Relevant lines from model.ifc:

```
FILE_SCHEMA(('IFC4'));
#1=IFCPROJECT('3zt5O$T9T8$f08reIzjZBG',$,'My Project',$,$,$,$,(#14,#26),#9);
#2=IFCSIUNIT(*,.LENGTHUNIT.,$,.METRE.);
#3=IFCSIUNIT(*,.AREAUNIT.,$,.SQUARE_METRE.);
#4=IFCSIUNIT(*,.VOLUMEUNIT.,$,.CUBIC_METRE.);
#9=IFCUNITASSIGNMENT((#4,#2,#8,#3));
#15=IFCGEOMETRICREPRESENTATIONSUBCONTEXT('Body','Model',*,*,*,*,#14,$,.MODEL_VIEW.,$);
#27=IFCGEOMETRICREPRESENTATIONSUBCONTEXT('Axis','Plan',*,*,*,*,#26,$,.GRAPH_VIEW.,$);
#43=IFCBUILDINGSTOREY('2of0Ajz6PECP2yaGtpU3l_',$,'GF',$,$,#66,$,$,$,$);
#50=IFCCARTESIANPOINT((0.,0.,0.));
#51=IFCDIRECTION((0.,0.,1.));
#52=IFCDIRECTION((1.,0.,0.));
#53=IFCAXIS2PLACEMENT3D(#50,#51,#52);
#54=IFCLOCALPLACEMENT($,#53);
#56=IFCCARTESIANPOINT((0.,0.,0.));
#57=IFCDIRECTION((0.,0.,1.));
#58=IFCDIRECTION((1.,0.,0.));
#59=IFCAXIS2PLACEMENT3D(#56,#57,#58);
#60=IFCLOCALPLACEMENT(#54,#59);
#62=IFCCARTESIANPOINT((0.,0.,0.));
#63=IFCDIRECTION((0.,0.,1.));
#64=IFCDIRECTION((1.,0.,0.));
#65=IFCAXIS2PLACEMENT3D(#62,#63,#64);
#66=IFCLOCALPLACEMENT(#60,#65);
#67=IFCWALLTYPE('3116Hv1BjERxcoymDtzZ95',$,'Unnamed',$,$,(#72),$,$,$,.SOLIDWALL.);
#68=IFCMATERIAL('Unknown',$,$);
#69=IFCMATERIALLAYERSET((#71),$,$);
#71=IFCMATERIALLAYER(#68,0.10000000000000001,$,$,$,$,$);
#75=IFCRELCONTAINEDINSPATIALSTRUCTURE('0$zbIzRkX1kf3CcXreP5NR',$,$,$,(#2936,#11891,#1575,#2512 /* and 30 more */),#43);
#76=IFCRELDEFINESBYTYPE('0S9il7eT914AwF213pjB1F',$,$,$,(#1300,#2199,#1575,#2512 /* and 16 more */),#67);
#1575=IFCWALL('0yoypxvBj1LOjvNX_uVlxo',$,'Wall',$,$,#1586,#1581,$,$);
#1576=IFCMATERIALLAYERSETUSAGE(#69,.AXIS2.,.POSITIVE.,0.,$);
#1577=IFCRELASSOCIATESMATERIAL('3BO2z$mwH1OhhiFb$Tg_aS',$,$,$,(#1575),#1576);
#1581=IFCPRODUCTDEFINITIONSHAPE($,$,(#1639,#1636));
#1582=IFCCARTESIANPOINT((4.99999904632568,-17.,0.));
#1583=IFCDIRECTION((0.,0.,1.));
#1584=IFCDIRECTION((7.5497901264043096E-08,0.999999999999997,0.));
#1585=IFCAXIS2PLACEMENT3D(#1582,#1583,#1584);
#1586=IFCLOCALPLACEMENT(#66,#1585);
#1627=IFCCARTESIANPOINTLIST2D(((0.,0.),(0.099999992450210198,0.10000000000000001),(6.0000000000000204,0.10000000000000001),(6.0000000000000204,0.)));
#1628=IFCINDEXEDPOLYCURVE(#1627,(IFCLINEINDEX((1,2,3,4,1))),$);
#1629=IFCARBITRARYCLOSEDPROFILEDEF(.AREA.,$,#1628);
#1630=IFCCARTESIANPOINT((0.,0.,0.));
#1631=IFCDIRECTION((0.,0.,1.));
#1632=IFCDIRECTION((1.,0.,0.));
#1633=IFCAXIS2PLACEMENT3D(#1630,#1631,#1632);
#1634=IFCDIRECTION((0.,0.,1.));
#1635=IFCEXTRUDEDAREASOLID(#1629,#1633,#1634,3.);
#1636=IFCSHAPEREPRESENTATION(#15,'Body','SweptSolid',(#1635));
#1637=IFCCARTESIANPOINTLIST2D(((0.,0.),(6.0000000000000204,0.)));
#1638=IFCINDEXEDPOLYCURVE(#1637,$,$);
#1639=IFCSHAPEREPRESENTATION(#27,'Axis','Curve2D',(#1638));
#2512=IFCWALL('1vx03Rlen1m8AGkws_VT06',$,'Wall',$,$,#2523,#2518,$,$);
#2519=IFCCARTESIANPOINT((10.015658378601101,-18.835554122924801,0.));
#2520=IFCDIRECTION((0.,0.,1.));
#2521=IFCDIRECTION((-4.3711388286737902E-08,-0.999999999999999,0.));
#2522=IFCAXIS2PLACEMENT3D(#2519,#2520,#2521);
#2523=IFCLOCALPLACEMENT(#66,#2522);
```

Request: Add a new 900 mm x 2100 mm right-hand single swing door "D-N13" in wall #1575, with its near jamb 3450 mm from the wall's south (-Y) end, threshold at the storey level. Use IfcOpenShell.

```python
import numpy as np
import ifcopenshell
import ifcopenshell.api.feature
import ifcopenshell.api.geometry
import ifcopenshell.api.root
import ifcopenshell.api.spatial
import ifcopenshell.geom
import ifcopenshell.util.element
import ifcopenshell.util.placement
import ifcopenshell.util.representation
import ifcopenshell.util.shape
import ifcopenshell.util.unit

model = ifcopenshell.open("model.ifc")
unit_scale = ifcopenshell.util.unit.calculate_unit_scale(model)
settings = ifcopenshell.geom.settings()


def volume(element):
    """Net volume in cubic metres, openings subtracted."""
    shape = ifcopenshell.geom.create_shape(settings, element)
    return ifcopenshell.util.shape.get_volume(shape.geometry)


wall = model.by_guid("0yoypxvBj1LOjvNX_uVlxo")
storey = ifcopenshell.util.element.get_container(wall, ifc_class="IfcBuildingStorey")
context = ifcopenshell.util.representation.get_context(model, "Model", "Body", "MODEL_VIEW")
before = volume(wall)

width, height, from_end, sill = 0.9, 2.1, 3.45, 0.0  # metres

# The wall runs along its own X axis, and the end named is its -X end.
wall_shape = ifcopenshell.geom.create_shape(settings, wall)
x, y, z = ifcopenshell.util.shape.get_vertices(wall_shape.geometry).T
start = x.min() + from_end
face, thickness = float(y.min()), float(y.max() - y.min())
wall_matrix = ifcopenshell.util.placement.get_local_placement(wall.ObjectPlacement)
level = ifcopenshell.util.placement.get_local_placement(storey.ObjectPlacement)[2, 3]


def in_wall(x, y):
    """Placement at x, y metres in the wall's axes, at sill height."""
    matrix = wall_matrix.copy()
    matrix[:, 3] = wall_matrix @ np.array([x / unit_scale, y / unit_scale, 0.0, 1.0])
    matrix[2, 3] = level + sill / unit_scale
    return matrix


# Opening: a box that overshoots both wall faces by 50 mm.
opening = ifcopenshell.api.root.create_entity(model, ifc_class="IfcOpeningElement", predefined_type="OPENING")
box = ifcopenshell.api.geometry.add_wall_representation(
    model, context=context, length=width, height=height, thickness=thickness + 0.1
)
ifcopenshell.api.geometry.assign_representation(model, product=opening, representation=box)
ifcopenshell.api.geometry.edit_object_placement(model, product=opening, matrix=in_wall(start, face - 0.05), is_si=False)
ifcopenshell.api.feature.add_feature(model, feature=opening, element=wall)

door = ifcopenshell.api.root.create_entity(model, ifc_class="IfcDoor", name="D-N13", predefined_type="DOOR")
door.OverallWidth, door.OverallHeight = width / unit_scale, height / unit_scale
door.OperationType = "SINGLE_SWING_RIGHT"
body = ifcopenshell.api.geometry.add_door_representation(
    model,
    context=context,
    overall_width=door.OverallWidth,
    overall_height=door.OverallHeight,
    operation_type="SINGLE_SWING_RIGHT",
    lining_properties={"LiningDepth": thickness / unit_scale, "ThresholdDepth": thickness / unit_scale},
)
ifcopenshell.api.geometry.assign_representation(model, product=door, representation=body)
ifcopenshell.api.spatial.assign_container(model, products=[door], relating_structure=storey)
ifcopenshell.api.feature.add_filling(model, opening=opening, element=door)

# The lining spans the wall, so the door starts at the wall face.
ifcopenshell.api.geometry.edit_object_placement(model, product=door, matrix=in_wall(start, face), is_si=False)

after = volume(wall)

print(f"wall volume {before:.3f} -> {after:.3f} m3")

model.write("model_v2.ifc")
```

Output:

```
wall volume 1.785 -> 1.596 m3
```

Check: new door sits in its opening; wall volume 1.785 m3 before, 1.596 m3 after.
